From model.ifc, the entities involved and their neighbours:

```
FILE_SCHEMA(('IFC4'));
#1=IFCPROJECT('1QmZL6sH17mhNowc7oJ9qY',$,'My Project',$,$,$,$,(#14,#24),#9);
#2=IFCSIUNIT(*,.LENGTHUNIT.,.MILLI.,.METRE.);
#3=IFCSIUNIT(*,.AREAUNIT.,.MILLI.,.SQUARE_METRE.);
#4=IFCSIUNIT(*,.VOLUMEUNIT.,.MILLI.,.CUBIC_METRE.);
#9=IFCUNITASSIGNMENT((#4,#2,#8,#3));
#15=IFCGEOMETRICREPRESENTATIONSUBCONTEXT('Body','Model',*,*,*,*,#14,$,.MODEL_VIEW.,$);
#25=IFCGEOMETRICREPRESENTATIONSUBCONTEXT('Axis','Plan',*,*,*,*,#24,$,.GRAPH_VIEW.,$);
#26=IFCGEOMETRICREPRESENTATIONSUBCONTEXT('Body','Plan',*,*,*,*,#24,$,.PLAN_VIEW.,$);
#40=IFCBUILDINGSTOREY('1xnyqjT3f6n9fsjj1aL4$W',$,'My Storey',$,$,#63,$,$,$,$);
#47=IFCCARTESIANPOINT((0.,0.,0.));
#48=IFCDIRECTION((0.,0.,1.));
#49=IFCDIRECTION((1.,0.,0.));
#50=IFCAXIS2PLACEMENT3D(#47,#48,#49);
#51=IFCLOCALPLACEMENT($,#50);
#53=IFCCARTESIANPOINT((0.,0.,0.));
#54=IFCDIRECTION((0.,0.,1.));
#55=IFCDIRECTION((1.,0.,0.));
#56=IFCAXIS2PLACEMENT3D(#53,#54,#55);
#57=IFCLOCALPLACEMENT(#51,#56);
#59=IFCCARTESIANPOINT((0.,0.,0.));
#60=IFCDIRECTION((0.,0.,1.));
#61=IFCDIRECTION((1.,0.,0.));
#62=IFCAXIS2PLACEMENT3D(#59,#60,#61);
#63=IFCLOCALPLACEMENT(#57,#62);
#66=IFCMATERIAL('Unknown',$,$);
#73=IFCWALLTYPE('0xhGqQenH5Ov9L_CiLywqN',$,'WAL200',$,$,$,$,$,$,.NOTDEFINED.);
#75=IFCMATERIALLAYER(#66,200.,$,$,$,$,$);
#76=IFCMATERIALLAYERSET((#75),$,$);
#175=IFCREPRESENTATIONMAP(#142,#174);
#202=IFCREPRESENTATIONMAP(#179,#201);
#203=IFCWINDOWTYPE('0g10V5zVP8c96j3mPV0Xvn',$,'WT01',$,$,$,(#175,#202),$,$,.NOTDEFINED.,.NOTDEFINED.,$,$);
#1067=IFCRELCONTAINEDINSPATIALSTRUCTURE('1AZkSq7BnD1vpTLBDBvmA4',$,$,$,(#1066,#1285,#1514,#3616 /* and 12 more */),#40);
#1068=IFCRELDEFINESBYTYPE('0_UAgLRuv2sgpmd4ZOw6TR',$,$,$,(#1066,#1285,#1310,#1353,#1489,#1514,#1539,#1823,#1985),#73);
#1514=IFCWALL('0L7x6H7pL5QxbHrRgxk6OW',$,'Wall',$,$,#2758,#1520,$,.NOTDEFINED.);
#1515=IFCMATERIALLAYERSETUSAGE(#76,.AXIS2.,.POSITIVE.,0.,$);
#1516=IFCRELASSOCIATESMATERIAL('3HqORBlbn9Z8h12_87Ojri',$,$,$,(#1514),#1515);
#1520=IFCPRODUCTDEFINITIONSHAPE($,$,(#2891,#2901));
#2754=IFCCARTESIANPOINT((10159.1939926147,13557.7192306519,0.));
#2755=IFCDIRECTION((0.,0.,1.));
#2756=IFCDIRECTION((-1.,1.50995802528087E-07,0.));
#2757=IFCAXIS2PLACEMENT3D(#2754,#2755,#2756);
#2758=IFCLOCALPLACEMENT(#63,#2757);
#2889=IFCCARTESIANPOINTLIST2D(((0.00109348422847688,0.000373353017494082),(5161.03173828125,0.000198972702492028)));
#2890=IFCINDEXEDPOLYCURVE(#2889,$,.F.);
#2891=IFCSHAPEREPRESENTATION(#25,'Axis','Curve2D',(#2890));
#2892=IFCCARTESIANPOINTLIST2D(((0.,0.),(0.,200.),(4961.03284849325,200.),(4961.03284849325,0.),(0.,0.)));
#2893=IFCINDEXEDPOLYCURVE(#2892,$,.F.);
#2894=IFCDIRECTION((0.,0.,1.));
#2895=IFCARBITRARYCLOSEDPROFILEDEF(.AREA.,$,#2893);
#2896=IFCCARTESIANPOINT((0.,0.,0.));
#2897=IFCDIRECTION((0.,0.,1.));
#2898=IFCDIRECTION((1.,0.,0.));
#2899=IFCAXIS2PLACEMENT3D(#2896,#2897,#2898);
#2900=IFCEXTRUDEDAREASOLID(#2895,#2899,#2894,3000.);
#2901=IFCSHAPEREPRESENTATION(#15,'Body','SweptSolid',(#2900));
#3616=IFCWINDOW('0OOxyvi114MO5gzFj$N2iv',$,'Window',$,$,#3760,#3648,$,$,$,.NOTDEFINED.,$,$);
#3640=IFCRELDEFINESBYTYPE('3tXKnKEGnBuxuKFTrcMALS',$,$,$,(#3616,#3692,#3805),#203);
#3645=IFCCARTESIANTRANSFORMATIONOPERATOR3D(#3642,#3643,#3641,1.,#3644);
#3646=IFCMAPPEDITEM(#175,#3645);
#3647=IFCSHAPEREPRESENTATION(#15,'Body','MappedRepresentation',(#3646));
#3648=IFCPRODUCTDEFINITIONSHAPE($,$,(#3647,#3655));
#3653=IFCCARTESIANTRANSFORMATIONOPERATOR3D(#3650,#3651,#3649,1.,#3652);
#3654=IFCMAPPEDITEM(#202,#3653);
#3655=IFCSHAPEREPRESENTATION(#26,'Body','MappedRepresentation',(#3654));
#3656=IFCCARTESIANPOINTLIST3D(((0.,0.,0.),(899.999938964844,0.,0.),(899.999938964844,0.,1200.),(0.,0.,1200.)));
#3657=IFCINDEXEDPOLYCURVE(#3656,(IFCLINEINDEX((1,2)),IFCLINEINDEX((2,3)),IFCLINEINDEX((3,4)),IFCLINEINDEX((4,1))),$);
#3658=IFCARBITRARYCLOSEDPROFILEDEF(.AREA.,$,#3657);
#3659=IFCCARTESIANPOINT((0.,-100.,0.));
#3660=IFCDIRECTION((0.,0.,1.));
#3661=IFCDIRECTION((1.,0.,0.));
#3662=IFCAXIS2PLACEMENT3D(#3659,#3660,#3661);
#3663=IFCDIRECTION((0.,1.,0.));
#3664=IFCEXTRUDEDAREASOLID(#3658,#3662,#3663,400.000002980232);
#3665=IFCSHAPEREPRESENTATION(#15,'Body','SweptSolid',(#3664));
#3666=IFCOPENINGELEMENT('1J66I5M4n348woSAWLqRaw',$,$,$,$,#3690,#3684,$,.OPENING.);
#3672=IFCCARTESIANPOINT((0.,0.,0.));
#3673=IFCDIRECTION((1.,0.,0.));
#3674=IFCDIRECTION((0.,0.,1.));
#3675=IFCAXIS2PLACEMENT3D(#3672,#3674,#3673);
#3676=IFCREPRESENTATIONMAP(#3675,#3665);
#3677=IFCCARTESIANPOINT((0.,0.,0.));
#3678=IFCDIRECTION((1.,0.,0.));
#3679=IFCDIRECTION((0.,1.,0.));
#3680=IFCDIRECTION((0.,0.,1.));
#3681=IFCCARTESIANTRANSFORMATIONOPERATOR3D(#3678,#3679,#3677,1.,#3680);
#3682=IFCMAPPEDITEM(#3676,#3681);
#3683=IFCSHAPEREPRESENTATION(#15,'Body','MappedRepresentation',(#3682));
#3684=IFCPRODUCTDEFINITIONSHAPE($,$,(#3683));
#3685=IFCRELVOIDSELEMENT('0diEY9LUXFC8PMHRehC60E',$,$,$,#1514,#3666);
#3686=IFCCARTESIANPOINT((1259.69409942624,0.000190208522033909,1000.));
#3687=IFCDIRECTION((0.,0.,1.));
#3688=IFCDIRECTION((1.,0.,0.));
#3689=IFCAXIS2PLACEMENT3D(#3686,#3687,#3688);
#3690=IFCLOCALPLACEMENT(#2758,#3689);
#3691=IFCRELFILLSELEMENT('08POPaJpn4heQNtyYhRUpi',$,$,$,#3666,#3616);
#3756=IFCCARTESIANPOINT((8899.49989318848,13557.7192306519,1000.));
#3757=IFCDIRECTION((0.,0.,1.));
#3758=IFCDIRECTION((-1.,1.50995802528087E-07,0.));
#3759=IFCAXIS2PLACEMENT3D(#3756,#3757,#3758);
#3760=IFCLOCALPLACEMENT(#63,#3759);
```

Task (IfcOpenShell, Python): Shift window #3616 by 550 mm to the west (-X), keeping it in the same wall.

```python
import ifcopenshell
import ifcopenshell.api.geometry
import ifcopenshell.util.placement
import ifcopenshell.util.unit

model = ifcopenshell.open("model.ifc")
unit_scale = ifcopenshell.util.unit.calculate_unit_scale(model)

window = model.by_id(3616)
opening = window.FillsVoids[0].RelatingOpeningElement
wall = opening.VoidsElements[0].RelatingBuildingElement

wall_matrix = ifcopenshell.util.placement.get_local_placement(wall.ObjectPlacement)
shift = wall_matrix[:3, 0] * 0.55 / unit_scale
before = ifcopenshell.util.placement.get_local_placement(window.ObjectPlacement)[:3, 3].copy()

# The window is not placed relative to its opening, so move both.
for product in (opening, window):
    matrix = ifcopenshell.util.placement.get_local_placement(product.ObjectPlacement)
    matrix[:3, 3] += shift
    ifcopenshell.api.geometry.edit_object_placement(model, product=product, matrix=matrix, is_si=False)

after = ifcopenshell.util.placement.get_local_placement(window.ObjectPlacement)[:3, 3]
print("window moved by", (after - before).round(3) + 0.0)

model.write("model_v2.ifc")
```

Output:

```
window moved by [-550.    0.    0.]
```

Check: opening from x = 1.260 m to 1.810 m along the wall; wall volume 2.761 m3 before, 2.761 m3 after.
